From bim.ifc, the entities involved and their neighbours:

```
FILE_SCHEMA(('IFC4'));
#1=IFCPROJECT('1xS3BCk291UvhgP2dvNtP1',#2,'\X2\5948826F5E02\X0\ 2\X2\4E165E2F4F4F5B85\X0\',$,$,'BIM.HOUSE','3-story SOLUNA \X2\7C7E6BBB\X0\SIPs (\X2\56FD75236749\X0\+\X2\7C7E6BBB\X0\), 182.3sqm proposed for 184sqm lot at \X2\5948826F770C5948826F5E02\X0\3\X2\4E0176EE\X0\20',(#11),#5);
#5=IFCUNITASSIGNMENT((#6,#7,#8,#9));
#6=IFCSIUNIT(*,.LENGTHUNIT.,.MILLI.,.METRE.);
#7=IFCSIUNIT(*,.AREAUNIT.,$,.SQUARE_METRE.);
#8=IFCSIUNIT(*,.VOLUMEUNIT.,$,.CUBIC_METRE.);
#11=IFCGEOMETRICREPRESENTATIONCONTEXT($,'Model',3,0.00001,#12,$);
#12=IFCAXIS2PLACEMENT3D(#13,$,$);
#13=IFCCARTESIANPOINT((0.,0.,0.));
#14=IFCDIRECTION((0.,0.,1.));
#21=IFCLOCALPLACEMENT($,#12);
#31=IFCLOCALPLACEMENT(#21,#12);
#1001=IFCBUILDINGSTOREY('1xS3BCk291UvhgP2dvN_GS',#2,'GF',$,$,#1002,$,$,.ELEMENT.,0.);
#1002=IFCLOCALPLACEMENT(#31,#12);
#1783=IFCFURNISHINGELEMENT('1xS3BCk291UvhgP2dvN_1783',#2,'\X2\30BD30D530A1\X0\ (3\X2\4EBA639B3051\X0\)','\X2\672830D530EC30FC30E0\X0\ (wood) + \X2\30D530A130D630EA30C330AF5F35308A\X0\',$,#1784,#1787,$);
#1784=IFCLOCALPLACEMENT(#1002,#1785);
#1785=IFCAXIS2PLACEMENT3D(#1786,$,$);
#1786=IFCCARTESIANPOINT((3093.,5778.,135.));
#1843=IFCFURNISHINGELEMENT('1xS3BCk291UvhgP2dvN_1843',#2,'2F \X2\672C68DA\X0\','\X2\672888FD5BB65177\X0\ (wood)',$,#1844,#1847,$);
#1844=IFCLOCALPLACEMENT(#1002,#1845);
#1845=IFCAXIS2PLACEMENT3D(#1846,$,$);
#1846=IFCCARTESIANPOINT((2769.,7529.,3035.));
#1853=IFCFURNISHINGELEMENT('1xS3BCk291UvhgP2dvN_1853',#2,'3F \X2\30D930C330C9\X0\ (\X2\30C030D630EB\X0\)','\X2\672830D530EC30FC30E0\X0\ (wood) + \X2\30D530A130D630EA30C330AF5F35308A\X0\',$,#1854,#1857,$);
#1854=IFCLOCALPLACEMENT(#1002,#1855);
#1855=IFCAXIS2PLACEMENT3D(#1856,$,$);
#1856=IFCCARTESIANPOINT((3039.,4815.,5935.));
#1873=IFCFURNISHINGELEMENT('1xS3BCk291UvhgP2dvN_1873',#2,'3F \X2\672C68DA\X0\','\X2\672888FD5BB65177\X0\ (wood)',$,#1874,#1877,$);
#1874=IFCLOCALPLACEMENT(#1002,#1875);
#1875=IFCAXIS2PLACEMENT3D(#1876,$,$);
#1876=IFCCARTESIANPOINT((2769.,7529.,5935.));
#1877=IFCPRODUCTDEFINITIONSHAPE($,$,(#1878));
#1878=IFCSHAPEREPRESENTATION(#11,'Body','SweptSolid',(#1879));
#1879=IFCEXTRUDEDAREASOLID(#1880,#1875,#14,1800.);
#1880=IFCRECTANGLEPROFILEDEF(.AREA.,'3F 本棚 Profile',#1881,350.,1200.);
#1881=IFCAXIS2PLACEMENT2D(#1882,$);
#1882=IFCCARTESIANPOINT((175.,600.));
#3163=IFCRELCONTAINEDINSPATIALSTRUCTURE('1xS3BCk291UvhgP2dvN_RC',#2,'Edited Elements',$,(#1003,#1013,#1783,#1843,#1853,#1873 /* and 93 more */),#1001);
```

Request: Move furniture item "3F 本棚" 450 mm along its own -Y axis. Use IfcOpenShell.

```python
import ifcopenshell
import ifcopenshell.api.geometry
import ifcopenshell.util.placement

model = ifcopenshell.open("bim.ifc")

item = model.by_guid("1xS3BCk291UvhgP2dvN_1873")
matrix = ifcopenshell.util.placement.get_local_placement(item.ObjectPlacement)
matrix[:3, 3] -= matrix[:3, 1] * 450.0
ifcopenshell.api.geometry.edit_object_placement(model, product=item, matrix=matrix, is_si=False)

print(ifcopenshell.util.placement.get_local_placement(item.ObjectPlacement).round(3) + 0.0)

model.write("bim_edited.ifc")
```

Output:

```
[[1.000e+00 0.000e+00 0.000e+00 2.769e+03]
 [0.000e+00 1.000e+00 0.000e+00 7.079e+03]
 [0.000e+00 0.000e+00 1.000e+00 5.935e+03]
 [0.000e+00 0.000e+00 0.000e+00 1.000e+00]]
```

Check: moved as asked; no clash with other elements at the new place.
